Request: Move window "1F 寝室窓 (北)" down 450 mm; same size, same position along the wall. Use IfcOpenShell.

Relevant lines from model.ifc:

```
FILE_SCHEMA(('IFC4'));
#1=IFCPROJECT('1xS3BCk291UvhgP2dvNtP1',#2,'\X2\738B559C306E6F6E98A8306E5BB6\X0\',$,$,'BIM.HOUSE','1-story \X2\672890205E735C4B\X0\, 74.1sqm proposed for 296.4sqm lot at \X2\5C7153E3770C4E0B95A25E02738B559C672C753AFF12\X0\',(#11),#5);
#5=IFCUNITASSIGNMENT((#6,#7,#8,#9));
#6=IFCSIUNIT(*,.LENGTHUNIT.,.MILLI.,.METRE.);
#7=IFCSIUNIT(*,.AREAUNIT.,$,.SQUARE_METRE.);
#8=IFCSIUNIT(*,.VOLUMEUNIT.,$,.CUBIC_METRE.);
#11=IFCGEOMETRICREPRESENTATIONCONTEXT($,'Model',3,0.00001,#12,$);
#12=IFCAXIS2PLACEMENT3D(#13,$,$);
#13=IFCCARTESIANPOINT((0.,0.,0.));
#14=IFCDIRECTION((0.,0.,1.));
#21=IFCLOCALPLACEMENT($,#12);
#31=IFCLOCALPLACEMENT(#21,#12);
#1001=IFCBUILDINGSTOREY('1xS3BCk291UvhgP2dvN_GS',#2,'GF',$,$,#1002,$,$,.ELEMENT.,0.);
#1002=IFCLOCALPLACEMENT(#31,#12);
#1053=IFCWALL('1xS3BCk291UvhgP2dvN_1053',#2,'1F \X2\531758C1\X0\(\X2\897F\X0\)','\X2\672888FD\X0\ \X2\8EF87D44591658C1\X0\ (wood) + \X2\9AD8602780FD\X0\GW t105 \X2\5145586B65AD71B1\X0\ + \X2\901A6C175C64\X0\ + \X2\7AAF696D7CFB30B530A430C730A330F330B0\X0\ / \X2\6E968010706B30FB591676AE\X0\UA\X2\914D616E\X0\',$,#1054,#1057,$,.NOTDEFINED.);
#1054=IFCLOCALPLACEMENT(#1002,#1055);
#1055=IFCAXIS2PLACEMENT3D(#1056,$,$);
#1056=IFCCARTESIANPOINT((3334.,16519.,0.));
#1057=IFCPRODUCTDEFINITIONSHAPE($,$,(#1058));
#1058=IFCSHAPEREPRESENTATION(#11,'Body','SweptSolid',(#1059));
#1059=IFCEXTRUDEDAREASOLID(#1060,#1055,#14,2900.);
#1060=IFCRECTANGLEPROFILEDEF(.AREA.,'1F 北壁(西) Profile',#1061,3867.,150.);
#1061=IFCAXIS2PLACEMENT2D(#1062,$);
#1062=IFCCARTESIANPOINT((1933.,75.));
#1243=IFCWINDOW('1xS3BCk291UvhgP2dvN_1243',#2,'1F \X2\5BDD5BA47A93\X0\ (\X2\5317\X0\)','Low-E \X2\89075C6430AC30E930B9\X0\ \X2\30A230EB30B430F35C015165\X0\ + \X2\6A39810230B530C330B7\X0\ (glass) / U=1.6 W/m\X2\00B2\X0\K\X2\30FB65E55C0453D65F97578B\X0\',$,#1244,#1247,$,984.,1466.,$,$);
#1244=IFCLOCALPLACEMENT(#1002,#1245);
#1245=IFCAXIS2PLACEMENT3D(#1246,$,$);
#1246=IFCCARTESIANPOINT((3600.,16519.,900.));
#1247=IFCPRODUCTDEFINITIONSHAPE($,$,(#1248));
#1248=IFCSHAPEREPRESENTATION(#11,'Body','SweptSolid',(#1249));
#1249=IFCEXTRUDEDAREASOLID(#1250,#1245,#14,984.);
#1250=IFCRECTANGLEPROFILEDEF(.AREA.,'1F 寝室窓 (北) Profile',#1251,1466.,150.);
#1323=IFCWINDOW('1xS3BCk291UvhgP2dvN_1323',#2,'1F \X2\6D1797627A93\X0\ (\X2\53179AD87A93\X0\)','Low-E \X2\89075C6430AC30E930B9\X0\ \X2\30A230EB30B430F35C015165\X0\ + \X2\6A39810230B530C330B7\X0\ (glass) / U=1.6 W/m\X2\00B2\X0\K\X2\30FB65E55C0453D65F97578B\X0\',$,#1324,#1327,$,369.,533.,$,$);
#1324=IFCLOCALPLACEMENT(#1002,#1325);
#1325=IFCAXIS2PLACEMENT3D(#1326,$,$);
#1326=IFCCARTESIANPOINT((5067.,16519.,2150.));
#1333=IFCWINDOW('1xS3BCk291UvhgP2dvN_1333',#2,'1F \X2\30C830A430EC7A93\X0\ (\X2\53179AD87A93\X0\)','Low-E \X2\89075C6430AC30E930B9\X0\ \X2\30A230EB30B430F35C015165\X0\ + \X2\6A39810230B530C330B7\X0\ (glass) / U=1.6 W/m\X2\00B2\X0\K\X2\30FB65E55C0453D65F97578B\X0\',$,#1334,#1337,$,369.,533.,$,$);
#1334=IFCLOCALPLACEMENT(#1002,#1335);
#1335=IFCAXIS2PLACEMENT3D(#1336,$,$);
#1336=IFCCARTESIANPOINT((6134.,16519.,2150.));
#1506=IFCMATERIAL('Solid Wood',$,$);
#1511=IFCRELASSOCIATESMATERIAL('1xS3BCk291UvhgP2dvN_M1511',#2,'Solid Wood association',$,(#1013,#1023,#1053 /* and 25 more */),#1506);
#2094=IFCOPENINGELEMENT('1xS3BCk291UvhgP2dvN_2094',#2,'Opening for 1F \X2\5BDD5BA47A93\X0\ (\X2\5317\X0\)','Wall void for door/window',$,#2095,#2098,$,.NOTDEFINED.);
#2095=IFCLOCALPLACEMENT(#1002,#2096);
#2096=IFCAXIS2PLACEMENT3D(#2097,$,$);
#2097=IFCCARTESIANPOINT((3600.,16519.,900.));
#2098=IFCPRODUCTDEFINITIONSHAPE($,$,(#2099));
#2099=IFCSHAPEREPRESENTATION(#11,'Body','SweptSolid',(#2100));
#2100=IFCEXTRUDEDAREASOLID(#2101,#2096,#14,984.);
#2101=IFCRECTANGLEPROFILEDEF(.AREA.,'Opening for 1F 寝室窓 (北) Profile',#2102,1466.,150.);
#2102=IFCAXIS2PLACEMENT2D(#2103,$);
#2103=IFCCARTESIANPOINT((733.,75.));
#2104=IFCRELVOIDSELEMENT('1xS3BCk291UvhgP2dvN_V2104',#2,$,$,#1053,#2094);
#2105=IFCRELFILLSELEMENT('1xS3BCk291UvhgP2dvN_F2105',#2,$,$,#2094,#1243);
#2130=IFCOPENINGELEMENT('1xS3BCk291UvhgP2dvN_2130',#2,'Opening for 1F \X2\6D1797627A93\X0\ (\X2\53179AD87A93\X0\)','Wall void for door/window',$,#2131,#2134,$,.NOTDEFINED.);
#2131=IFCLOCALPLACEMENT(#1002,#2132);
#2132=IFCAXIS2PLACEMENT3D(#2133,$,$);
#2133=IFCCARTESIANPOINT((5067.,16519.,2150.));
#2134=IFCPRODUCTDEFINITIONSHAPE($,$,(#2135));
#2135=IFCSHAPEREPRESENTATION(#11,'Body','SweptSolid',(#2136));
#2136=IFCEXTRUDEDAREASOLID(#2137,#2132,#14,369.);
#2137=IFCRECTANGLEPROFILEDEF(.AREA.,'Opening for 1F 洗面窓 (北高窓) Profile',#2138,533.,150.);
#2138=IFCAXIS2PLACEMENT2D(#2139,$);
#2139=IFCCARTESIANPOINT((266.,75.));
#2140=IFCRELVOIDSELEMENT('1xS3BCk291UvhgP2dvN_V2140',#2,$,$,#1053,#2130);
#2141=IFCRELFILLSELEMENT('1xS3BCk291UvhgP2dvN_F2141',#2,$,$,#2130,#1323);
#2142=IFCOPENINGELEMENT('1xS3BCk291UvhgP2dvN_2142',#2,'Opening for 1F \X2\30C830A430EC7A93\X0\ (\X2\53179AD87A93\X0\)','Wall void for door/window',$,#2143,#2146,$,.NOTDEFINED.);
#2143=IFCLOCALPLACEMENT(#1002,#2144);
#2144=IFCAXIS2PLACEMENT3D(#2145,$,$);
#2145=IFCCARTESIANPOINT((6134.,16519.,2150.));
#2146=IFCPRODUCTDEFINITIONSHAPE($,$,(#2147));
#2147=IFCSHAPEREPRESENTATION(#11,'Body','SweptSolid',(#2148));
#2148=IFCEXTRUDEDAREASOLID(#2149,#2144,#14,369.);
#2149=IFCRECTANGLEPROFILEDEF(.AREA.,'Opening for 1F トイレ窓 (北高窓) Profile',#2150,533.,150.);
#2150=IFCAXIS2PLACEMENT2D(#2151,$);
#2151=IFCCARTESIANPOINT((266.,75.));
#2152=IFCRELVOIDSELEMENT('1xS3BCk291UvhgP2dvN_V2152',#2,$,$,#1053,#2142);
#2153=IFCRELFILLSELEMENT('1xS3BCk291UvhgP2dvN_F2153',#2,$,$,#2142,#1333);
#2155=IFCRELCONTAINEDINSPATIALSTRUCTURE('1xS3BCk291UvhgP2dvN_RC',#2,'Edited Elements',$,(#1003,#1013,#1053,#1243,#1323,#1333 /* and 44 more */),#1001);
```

```python
import numpy as np
import ifcopenshell
import ifcopenshell.api.geometry
import ifcopenshell.util.placement
import ifcopenshell.util.unit

model = ifcopenshell.open("model.ifc")
unit_scale = ifcopenshell.util.unit.calculate_unit_scale(model)

window = model.by_id(1243)
opening = window.FillsVoids[0].RelatingOpeningElement
dz = -450.0

shift = np.array([0.0, 0.0, dz])
# The window is not placed relative to its opening, so move both.
for product in (opening, window):
    matrix = ifcopenshell.util.placement.get_local_placement(product.ObjectPlacement)
    matrix[:3, 3] += shift
    ifcopenshell.api.geometry.edit_object_placement(model, product=product, matrix=matrix, is_si=False)

print(f"moved by {dz * unit_scale:+.3f} m")

model.write("model_updated.ifc")
```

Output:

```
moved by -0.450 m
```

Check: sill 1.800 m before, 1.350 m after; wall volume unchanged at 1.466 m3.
